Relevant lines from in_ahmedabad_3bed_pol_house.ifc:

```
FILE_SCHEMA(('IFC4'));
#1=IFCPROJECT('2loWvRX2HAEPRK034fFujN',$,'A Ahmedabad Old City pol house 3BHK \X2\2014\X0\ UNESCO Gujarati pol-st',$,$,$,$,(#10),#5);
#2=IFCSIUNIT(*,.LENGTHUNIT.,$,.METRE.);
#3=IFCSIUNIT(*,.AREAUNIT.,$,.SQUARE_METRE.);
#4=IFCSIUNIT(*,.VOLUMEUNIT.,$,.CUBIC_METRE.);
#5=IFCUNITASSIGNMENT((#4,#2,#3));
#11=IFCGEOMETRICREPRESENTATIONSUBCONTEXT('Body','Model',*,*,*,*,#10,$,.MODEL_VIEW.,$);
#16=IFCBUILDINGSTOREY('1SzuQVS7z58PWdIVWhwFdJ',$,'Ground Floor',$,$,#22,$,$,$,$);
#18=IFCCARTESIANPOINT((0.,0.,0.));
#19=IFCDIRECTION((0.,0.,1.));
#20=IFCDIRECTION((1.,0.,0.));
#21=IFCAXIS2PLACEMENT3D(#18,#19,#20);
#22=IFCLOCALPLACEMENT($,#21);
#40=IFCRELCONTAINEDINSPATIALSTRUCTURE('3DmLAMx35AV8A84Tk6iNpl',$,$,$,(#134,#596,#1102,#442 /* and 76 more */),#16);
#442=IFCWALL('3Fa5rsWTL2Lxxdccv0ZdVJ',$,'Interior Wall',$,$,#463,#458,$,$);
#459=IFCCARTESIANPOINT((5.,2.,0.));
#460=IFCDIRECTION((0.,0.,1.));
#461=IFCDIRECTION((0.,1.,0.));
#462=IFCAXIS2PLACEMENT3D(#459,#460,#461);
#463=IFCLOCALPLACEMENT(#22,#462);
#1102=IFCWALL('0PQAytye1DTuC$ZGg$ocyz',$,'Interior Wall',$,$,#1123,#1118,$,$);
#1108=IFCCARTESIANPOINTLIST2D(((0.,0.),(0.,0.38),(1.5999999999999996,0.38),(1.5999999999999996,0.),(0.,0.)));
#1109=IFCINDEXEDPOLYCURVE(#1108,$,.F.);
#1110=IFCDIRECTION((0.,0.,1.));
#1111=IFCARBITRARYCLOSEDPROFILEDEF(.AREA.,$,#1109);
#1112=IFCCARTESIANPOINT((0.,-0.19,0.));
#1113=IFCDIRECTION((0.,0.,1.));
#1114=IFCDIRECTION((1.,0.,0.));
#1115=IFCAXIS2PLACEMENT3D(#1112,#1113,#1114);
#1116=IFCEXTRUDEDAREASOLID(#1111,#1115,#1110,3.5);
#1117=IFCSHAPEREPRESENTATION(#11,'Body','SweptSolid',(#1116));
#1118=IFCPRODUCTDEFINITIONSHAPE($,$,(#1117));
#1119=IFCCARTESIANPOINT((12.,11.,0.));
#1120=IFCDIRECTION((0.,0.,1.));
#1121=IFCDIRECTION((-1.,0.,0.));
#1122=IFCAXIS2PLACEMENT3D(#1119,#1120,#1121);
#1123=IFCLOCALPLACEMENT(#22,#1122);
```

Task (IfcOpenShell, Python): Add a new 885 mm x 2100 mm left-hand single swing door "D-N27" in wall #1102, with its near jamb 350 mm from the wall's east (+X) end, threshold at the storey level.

```python
import numpy as np
import ifcopenshell
import ifcopenshell.api.feature
import ifcopenshell.api.geometry
import ifcopenshell.api.root
import ifcopenshell.api.spatial
import ifcopenshell.geom
import ifcopenshell.util.element
import ifcopenshell.util.placement
import ifcopenshell.util.representation
import ifcopenshell.util.shape
import ifcopenshell.util.unit

model = ifcopenshell.open("in_ahmedabad_3bed_pol_house.ifc")
unit_scale = ifcopenshell.util.unit.calculate_unit_scale(model)
settings = ifcopenshell.geom.settings()


def volume(element):
    """Net volume in cubic metres, openings subtracted."""
    shape = ifcopenshell.geom.create_shape(settings, element)
    return ifcopenshell.util.shape.get_volume(shape.geometry)


wall = model.by_id(1102)
storey = ifcopenshell.util.element.get_container(wall, ifc_class="IfcBuildingStorey")
context = ifcopenshell.util.representation.get_context(model, "Model", "Body", "MODEL_VIEW")
before = volume(wall)

width, height, from_end, sill = 0.885, 2.1, 0.35, 0.0  # metres

# The wall runs along its own X axis, and the end named is its -X end.
wall_shape = ifcopenshell.geom.create_shape(settings, wall)
x, y, z = ifcopenshell.util.shape.get_vertices(wall_shape.geometry).T
start = x.min() + from_end
face, thickness = float(y.min()), float(y.max() - y.min())
wall_matrix = ifcopenshell.util.placement.get_local_placement(wall.ObjectPlacement)
level = ifcopenshell.util.placement.get_local_placement(storey.ObjectPlacement)[2, 3]


def in_wall(x, y):
    """Placement at x, y metres in the wall's axes, at sill height."""
    matrix = wall_matrix.copy()
    matrix[:, 3] = wall_matrix @ np.array([x / unit_scale, y / unit_scale, 0.0, 1.0])
    matrix[2, 3] = level + sill / unit_scale
    return matrix


# Opening: a box that overshoots both wall faces by 50 mm.
opening = ifcopenshell.api.root.create_entity(model, ifc_class="IfcOpeningElement", predefined_type="OPENING")
box = ifcopenshell.api.geometry.add_wall_representation(
    model, context=context, length=width, height=height, thickness=thickness + 0.1
)
ifcopenshell.api.geometry.assign_representation(model, product=opening, representation=box)
ifcopenshell.api.geometry.edit_object_placement(model, product=opening, matrix=in_wall(start, face - 0.05), is_si=False)
ifcopenshell.api.feature.add_feature(model, feature=opening, element=wall)

door = ifcopenshell.api.root.create_entity(model, ifc_class="IfcDoor", name="D-N27", predefined_type="DOOR")
door.OverallWidth, door.OverallHeight = width / unit_scale, height / unit_scale
door.OperationType = "SINGLE_SWING_LEFT"
body = ifcopenshell.api.geometry.add_door_representation(
    model,
    context=context,
    overall_width=door.OverallWidth,
    overall_height=door.OverallHeight,
    operation_type="SINGLE_SWING_LEFT",
    lining_properties={"LiningDepth": thickness / unit_scale, "ThresholdDepth": thickness / unit_scale},
)
ifcopenshell.api.geometry.assign_representation(model, product=door, representation=body)
ifcopenshell.api.spatial.assign_container(model, products=[door], relating_structure=storey)
ifcopenshell.api.feature.add_filling(model, opening=opening, element=door)

# The lining spans the wall, so the door starts at the wall face.
ifcopenshell.api.geometry.edit_object_placement(model, product=door, matrix=in_wall(start, face), is_si=False)

after = volume(wall)

print(f"wall volume {before:.3f} -> {after:.3f} m3")

model.write("in_ahmedabad_3bed_pol_house_updated.ifc")
```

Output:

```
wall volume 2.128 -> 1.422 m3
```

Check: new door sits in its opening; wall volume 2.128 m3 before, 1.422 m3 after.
